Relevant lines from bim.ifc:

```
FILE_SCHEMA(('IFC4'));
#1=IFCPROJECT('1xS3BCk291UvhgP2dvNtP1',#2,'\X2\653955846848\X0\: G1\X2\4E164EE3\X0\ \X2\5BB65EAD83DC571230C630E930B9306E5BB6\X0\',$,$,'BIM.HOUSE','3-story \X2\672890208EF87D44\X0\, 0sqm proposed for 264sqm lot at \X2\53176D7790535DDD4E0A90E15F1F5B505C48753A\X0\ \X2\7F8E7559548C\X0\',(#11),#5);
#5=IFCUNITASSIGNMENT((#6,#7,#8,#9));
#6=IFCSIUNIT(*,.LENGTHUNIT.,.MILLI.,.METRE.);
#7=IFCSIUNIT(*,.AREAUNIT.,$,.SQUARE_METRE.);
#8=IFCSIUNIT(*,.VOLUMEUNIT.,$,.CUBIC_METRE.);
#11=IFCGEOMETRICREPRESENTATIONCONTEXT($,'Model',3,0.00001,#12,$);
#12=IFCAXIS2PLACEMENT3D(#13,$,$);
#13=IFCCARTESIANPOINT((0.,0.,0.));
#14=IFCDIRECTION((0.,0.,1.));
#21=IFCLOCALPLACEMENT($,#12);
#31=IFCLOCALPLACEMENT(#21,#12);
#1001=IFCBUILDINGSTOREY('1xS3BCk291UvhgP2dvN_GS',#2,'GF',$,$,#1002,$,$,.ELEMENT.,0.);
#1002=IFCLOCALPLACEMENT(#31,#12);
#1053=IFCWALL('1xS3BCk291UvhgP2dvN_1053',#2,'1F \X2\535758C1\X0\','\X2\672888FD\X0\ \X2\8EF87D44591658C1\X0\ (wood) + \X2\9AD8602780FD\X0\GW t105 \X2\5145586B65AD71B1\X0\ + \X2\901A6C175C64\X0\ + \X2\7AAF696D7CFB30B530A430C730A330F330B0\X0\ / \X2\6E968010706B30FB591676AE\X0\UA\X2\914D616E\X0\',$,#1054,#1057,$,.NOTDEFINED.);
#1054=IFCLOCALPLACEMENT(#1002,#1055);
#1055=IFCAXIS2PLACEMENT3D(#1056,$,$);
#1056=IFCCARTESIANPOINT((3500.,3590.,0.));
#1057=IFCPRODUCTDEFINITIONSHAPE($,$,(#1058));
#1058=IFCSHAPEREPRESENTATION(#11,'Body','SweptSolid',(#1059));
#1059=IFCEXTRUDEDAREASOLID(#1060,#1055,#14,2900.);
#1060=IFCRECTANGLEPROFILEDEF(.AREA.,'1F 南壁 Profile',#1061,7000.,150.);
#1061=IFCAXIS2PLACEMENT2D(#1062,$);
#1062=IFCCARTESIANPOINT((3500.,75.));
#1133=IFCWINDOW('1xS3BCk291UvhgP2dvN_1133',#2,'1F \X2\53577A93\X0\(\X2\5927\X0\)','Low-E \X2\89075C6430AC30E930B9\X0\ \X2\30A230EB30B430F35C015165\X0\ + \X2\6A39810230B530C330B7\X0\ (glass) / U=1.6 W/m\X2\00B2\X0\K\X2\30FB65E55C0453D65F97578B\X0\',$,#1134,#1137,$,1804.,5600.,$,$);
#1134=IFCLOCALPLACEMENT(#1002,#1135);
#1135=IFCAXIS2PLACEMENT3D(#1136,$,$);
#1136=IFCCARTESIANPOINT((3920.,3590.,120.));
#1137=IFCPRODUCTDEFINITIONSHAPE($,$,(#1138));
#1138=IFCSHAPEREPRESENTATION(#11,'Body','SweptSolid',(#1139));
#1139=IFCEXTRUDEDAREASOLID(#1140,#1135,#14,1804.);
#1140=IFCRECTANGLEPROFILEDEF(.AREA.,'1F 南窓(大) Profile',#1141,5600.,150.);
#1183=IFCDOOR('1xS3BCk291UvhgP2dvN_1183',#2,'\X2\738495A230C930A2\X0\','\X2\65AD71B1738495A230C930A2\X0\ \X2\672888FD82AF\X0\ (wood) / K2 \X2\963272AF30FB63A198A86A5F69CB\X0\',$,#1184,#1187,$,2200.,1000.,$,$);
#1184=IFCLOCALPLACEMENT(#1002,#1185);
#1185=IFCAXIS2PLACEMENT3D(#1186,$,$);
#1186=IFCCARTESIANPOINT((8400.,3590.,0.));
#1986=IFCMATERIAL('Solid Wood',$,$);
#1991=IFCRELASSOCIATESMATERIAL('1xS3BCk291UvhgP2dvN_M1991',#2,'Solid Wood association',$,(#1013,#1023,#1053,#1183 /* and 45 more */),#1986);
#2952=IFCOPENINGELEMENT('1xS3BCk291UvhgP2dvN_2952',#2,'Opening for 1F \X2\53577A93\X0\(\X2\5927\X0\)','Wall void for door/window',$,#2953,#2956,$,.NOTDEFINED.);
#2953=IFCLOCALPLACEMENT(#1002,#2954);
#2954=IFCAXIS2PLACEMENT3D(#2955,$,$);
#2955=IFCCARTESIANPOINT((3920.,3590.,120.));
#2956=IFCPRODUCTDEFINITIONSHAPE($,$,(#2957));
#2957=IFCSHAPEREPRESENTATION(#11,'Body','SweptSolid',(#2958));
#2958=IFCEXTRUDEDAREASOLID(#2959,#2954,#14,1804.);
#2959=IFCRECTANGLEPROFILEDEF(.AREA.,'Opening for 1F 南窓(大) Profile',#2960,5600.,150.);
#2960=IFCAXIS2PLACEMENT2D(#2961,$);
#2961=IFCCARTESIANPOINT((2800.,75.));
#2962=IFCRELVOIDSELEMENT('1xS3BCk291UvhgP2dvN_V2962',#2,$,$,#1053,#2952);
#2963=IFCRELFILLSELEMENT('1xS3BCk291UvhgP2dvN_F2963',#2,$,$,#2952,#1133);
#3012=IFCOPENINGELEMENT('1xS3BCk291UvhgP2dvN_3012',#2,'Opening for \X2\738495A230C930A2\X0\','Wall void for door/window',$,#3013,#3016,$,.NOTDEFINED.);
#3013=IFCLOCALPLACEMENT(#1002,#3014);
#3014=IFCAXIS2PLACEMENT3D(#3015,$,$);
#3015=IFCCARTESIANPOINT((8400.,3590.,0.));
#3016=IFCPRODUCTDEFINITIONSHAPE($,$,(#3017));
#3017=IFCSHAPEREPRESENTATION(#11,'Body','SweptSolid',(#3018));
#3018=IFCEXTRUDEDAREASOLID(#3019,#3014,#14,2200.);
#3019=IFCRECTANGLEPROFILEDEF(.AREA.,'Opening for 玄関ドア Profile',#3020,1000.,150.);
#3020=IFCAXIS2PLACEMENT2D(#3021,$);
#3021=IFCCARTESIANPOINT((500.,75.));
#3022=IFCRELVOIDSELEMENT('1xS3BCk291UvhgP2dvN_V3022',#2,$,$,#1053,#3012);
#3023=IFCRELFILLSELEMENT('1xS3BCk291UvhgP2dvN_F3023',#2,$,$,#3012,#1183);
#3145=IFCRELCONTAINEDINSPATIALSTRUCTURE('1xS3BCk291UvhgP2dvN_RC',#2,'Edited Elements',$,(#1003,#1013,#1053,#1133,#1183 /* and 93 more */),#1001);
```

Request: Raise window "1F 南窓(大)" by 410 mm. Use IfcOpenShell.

```python
import numpy as np
import ifcopenshell
import ifcopenshell.api.geometry
import ifcopenshell.util.placement
import ifcopenshell.util.unit

model = ifcopenshell.open("bim.ifc")
unit_scale = ifcopenshell.util.unit.calculate_unit_scale(model)

window = model.by_guid("1xS3BCk291UvhgP2dvN_1133")
opening = window.FillsVoids[0].RelatingOpeningElement
dz = 0.41 / unit_scale

shift = np.array([0.0, 0.0, dz])
# The window is not placed relative to its opening, so move both.
for product in (opening, window):
    matrix = ifcopenshell.util.placement.get_local_placement(product.ObjectPlacement)
    matrix[:3, 3] += shift
    ifcopenshell.api.geometry.edit_object_placement(model, product=product, matrix=matrix, is_si=False)

print(f"moved by {dz * unit_scale:+.3f} m")

model.write("bim_v2.ifc")
```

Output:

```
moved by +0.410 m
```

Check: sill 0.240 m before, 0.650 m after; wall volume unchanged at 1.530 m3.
